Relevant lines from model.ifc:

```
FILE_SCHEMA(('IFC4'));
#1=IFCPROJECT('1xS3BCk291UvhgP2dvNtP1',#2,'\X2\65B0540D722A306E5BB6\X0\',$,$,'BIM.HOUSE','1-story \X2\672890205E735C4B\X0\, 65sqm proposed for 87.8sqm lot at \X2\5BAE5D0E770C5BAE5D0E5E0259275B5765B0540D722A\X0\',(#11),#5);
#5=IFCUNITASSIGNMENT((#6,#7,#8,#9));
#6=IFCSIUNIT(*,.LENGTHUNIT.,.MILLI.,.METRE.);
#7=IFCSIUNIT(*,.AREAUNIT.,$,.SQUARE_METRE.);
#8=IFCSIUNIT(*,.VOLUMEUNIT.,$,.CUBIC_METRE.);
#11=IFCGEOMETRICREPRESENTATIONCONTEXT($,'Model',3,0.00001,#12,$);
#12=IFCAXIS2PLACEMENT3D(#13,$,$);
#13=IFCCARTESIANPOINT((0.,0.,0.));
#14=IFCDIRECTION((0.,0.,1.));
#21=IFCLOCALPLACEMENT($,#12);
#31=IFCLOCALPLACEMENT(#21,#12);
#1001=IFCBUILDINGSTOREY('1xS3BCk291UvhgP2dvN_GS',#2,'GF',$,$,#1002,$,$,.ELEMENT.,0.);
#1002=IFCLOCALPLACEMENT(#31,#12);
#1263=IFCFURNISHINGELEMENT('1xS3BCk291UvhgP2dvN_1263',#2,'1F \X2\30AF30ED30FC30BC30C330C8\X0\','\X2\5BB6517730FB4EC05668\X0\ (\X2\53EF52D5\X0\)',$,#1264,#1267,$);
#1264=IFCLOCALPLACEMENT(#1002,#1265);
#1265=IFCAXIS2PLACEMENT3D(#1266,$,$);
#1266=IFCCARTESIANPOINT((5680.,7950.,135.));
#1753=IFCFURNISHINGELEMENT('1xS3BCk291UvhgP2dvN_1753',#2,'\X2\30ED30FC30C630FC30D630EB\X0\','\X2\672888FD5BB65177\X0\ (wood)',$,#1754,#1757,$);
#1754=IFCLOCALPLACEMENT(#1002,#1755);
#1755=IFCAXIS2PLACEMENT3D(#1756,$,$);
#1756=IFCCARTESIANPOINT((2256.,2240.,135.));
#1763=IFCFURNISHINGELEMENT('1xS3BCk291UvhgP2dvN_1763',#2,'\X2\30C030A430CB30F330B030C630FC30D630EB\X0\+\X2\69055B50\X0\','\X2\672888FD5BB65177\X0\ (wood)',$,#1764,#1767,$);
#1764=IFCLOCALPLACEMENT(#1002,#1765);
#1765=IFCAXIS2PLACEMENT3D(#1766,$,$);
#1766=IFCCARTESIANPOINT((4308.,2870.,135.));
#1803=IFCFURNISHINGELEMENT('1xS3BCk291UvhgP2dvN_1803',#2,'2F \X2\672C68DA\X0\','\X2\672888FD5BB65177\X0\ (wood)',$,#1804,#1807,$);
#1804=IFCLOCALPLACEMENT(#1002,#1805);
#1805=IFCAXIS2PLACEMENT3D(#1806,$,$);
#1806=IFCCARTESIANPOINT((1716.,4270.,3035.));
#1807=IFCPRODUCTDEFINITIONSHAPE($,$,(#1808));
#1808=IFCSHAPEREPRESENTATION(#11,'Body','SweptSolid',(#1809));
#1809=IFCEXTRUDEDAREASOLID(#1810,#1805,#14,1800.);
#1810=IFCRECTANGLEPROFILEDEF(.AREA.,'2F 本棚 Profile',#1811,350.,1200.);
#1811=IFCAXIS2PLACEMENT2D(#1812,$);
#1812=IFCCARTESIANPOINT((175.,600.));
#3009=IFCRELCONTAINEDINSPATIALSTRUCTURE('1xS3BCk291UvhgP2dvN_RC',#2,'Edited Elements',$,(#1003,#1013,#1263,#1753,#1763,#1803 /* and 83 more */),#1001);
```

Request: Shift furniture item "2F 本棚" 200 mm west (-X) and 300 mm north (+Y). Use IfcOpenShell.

```python
import ifcopenshell
import ifcopenshell.api.geometry
import ifcopenshell.util.placement

model = ifcopenshell.open("model.ifc")

item = model.by_guid("1xS3BCk291UvhgP2dvN_1803")
matrix = ifcopenshell.util.placement.get_local_placement(item.ObjectPlacement)
matrix[0, 3] -= 200.0
matrix[1, 3] += 300.0
ifcopenshell.api.geometry.edit_object_placement(model, product=item, matrix=matrix, is_si=False)

print(ifcopenshell.util.placement.get_local_placement(item.ObjectPlacement).round(3) + 0.0)

model.write("model_v2.ifc")
```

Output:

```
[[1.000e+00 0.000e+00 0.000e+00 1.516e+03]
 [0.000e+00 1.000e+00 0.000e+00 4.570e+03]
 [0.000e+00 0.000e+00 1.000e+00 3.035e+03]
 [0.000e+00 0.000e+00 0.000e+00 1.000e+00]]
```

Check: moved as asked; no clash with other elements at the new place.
